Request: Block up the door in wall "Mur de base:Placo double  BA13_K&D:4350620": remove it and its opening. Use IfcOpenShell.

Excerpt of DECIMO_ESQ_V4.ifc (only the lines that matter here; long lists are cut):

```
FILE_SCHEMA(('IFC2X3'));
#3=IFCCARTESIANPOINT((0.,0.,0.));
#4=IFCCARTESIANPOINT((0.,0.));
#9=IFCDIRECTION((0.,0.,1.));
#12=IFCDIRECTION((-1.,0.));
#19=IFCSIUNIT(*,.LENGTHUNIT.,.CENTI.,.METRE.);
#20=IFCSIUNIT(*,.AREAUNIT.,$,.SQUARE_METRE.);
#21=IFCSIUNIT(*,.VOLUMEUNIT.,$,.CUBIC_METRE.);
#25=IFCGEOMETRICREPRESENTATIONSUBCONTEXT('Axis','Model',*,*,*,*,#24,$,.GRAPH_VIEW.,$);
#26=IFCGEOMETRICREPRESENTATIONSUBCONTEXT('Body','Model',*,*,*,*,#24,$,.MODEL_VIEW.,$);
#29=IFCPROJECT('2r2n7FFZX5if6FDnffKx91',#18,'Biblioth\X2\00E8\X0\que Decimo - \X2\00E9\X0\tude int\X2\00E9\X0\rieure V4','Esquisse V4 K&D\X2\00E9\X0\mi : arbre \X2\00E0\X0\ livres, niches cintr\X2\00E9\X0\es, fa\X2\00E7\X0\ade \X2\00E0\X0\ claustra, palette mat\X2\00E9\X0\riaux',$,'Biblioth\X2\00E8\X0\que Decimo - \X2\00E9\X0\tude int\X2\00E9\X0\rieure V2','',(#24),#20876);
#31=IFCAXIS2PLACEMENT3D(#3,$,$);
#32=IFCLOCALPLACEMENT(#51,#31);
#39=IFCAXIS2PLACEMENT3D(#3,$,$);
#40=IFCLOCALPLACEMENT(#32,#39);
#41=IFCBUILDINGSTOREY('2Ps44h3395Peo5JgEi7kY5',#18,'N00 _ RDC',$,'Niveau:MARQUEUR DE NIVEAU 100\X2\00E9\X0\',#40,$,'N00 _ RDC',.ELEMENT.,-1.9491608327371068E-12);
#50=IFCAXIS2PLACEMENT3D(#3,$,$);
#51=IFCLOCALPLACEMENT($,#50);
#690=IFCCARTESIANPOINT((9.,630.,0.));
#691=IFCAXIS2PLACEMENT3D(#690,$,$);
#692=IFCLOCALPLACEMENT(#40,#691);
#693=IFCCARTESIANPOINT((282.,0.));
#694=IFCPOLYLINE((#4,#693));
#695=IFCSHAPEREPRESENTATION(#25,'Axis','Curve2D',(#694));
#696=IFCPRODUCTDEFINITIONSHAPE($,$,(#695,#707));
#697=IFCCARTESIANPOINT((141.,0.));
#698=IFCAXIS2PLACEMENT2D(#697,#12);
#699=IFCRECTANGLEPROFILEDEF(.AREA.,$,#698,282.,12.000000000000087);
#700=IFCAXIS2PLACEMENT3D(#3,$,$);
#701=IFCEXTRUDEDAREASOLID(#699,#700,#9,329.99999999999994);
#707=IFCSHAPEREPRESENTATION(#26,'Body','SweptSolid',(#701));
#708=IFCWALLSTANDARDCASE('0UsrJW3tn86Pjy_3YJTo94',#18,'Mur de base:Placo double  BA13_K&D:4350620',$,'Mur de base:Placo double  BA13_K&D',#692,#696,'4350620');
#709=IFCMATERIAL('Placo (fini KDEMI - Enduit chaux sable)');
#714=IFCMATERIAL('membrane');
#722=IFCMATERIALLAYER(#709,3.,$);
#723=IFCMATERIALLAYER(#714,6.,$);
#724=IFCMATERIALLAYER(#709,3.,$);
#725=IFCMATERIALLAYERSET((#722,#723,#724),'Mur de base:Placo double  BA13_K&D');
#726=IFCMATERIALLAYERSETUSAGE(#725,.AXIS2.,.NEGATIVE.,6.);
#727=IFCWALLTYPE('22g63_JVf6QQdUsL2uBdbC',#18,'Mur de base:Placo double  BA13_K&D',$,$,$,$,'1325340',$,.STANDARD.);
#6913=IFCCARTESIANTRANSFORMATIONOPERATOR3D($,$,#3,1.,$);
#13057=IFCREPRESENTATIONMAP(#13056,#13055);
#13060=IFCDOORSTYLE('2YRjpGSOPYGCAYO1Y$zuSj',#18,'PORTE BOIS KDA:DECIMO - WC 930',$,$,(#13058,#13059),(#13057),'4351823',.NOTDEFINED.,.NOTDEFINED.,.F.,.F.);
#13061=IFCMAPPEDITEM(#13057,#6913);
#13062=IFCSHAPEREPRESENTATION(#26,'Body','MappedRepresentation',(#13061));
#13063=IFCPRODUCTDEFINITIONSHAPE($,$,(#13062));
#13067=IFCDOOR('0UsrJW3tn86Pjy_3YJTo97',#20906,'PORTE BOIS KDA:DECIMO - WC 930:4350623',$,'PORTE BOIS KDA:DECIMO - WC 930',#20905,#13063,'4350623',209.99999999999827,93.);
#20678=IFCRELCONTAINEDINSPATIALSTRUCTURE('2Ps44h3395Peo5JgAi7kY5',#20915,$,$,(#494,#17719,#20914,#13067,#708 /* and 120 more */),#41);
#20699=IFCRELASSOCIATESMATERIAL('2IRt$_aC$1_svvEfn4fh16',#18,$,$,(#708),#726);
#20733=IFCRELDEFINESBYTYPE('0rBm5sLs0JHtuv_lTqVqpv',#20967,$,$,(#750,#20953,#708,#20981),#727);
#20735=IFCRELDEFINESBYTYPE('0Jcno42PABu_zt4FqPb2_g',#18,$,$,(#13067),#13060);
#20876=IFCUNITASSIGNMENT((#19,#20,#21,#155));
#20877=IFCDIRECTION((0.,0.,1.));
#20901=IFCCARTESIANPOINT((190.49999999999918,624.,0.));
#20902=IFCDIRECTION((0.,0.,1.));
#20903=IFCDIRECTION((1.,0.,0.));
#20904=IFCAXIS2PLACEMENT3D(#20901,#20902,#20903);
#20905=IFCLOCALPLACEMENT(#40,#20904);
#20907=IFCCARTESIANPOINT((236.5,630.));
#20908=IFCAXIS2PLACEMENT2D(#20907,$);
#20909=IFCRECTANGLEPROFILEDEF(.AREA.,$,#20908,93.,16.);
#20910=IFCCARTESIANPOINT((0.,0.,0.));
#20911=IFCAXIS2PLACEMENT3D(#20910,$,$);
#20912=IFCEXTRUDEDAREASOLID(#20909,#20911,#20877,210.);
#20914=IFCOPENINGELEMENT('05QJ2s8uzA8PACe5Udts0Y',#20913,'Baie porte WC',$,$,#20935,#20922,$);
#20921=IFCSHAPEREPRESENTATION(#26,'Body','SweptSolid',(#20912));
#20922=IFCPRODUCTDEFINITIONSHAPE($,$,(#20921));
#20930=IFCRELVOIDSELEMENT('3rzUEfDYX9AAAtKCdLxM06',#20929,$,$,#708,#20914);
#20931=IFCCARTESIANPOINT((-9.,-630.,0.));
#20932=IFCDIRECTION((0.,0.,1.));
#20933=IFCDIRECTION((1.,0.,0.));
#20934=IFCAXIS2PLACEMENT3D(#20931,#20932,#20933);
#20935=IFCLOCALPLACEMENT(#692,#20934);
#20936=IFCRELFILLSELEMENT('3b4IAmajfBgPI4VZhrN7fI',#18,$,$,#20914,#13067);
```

```python
import ifcopenshell
import ifcopenshell.api.feature
import ifcopenshell.api.root
import ifcopenshell.geom
import ifcopenshell.util.shape

model = ifcopenshell.open("DECIMO_ESQ_V4.ifc")
settings = ifcopenshell.geom.settings()


def volume(element):
    """Net volume in cubic metres, openings subtracted."""
    shape = ifcopenshell.geom.create_shape(settings, element)
    return ifcopenshell.util.shape.get_volume(shape.geometry)


door = model.by_guid("0UsrJW3tn86Pjy_3YJTo97")
opening = door.FillsVoids[0].RelatingOpeningElement
wall = opening.VoidsElements[0].RelatingBuildingElement
before = volume(wall)

ifcopenshell.api.root.remove_product(model, product=door)
ifcopenshell.api.feature.remove_feature(model, feature=opening)

after = volume(wall)

print(f"wall volume {before:.3f} -> {after:.3f} m3")

model.write("DECIMO_ESQ_V4_updated.ifc")
```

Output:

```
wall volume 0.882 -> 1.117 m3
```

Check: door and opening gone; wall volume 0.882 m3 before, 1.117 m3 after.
